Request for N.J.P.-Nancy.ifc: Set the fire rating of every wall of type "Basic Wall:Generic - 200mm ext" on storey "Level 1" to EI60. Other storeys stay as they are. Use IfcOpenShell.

First a look at what the model holds.

```python
import ifcopenshell
import ifcopenshell.util.element

model = ifcopenshell.open("N.J.P.-Nancy.ifc")
print(model.schema)
storey = next(s for s in model.by_type("IfcBuildingStorey") if s.Name == "Level 1")
walls = [e for e in ifcopenshell.util.element.get_decomposition(storey) if e.is_a("IfcWall")]
seen = {}
for e in walls:
    element_type = ifcopenshell.util.element.get_type(e)
    key = (element_type.Name if element_type != e and element_type else None, ifcopenshell.util.element.get_pset(e, "Pset_WallCommon", "FireRating"))
    seen[key] = seen.get(key, 0) + 1
for (name, value), count in sorted(seen.items(), key=str):
    print(count, "x", name, "|", value)
```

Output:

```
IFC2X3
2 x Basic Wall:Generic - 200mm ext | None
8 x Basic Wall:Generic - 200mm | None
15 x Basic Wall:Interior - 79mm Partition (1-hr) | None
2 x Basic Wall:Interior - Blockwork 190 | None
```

```python
import ifcopenshell
import ifcopenshell.api.pset
import ifcopenshell.util.element

model = ifcopenshell.open("N.J.P.-Nancy.ifc")

storey = next(s for s in model.by_type("IfcBuildingStorey") if s.Name == "Level 1")
walls = [e for e in ifcopenshell.util.element.get_decomposition(storey) if e.is_a("IfcWall")]

count = 0
for e in walls:
    element_type = ifcopenshell.util.element.get_type(e)
    if element_type in (None, e) or element_type.Name != "Basic Wall:Generic - 200mm ext":
        continue
    # add_pset returns the element's existing set when there is one.
    pset = ifcopenshell.api.pset.add_pset(model, product=e, name="Pset_WallCommon")
    ifcopenshell.api.pset.edit_pset(model, pset=pset, properties={"FireRating": "EI60"})
    count += 1

print(count, "walls updated")

model.write("N.J.P.-Nancy_v2.ifc")
```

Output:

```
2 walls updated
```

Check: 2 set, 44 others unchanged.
